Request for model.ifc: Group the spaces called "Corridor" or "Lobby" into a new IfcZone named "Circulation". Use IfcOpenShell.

First a look at what the model holds.

```python
import ifcopenshell

model = ifcopenshell.open("model.ifc")
print(model.schema)
seen = {}
for space in model.by_type("IfcSpace"):
    seen[space.LongName] = seen.get(space.LongName, 0) + 1
for name, count in sorted(seen.items(), key=str):
    print(count, "x", name)
print("zones:", [z.Name for z in model.by_type("IfcZone")][:20])
```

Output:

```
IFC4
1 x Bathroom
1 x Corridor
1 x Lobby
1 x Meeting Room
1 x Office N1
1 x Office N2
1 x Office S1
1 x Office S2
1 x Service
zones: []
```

```python
import ifcopenshell
import ifcopenshell.api.group
import ifcopenshell.api.root

model = ifcopenshell.open("model.ifc")

names = {"Corridor", "Lobby"}
spaces = [s for s in model.by_type("IfcSpace") if s.LongName in names]

zone = ifcopenshell.api.root.create_entity(model, ifc_class="IfcZone", name="Circulation")
ifcopenshell.api.group.assign_group(model, products=spaces, group=zone)
print(len(spaces), "spaces in", zone.Name)

model.write("model_edited.ifc")
```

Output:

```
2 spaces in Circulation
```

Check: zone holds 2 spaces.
